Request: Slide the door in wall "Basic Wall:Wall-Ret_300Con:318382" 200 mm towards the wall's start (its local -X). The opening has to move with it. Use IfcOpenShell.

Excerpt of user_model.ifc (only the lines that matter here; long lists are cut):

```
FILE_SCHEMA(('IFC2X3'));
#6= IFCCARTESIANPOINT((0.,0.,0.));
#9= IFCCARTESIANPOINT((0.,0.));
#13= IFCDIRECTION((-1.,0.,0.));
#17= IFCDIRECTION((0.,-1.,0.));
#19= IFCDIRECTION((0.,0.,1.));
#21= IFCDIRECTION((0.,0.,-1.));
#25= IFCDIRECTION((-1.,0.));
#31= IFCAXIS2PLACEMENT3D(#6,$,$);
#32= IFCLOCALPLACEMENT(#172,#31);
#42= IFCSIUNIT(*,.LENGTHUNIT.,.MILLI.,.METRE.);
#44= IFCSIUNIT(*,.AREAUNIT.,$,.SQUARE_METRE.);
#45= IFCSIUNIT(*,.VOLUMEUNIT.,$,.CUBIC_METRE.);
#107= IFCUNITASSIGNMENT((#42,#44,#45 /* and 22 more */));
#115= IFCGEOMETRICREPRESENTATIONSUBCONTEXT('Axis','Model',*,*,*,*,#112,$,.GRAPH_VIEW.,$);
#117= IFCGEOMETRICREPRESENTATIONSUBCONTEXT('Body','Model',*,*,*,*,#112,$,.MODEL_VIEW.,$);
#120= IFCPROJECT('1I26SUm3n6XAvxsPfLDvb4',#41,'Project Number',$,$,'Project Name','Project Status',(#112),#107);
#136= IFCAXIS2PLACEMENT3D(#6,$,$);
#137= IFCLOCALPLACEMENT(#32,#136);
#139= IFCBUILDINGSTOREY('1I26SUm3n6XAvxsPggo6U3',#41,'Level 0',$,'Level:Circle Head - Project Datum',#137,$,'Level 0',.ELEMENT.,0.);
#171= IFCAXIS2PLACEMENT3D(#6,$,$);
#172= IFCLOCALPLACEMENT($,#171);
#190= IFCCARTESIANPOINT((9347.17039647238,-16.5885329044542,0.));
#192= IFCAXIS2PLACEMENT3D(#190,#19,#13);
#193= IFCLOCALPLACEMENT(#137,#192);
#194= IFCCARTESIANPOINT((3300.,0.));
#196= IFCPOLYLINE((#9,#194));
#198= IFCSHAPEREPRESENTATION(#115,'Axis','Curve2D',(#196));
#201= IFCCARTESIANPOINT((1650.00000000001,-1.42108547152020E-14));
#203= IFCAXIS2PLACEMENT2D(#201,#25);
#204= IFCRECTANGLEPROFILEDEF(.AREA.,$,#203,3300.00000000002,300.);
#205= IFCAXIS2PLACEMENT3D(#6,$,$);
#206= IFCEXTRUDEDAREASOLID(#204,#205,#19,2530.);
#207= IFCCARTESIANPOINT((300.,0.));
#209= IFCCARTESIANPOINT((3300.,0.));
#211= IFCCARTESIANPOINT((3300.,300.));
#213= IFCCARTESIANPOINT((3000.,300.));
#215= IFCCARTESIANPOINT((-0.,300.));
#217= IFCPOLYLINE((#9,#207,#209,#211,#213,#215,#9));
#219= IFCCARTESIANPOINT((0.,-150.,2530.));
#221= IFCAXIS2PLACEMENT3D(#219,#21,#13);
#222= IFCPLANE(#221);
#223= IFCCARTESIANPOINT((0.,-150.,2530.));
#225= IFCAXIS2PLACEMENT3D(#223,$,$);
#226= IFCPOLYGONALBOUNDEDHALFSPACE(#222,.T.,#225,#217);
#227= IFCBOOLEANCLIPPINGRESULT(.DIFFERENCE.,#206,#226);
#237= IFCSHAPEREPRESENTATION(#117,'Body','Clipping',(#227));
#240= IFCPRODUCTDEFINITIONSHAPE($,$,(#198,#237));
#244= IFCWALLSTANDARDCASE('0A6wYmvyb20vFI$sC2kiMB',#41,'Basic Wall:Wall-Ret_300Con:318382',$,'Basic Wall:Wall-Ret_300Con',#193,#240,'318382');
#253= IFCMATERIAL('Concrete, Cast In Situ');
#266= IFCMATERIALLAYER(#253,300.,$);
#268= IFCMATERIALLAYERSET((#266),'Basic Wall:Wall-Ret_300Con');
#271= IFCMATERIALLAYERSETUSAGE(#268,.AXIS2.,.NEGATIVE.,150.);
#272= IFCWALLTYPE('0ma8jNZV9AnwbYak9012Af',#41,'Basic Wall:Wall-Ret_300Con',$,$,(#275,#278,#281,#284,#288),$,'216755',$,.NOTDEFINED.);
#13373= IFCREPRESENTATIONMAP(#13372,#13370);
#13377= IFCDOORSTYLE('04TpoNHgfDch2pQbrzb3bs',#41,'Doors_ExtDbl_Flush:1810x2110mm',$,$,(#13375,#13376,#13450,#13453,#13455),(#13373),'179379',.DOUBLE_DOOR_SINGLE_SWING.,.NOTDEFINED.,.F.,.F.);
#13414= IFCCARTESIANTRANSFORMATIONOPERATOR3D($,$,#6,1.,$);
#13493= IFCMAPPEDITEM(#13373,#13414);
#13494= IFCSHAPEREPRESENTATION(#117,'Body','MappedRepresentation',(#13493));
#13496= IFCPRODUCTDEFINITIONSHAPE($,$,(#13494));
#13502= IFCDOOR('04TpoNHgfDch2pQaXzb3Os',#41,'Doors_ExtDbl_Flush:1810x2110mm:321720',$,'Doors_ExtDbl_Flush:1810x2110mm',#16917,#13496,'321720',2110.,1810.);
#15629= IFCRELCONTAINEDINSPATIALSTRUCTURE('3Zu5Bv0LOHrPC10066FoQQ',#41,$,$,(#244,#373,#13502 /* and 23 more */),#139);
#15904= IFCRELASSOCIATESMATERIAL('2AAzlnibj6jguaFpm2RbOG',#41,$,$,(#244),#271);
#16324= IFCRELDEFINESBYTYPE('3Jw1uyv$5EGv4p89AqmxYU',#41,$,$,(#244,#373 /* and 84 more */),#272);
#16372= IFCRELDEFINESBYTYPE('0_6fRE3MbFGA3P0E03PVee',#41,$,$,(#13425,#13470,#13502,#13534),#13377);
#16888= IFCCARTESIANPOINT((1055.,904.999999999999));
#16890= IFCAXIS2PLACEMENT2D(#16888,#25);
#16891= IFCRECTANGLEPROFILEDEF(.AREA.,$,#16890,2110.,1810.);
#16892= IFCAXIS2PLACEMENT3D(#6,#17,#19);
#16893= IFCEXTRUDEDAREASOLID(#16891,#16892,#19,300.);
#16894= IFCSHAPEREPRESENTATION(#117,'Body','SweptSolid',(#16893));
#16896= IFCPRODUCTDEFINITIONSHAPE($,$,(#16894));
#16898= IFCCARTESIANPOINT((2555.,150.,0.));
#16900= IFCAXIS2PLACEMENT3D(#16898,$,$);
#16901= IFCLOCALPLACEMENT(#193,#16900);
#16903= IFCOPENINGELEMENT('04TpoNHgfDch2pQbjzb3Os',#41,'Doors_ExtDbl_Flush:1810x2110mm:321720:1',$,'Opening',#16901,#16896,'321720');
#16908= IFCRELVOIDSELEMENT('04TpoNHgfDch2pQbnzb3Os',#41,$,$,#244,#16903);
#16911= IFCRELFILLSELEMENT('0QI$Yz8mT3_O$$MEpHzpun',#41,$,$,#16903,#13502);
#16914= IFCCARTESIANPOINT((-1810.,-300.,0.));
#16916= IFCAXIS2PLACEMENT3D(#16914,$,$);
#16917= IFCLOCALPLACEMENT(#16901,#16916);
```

```python
import ifcopenshell
import ifcopenshell.api.geometry
import ifcopenshell.util.placement
import ifcopenshell.util.unit

model = ifcopenshell.open("user_model.ifc")
unit_scale = ifcopenshell.util.unit.calculate_unit_scale(model)

door = model.by_id(13502)
opening = door.FillsVoids[0].RelatingOpeningElement
wall = opening.VoidsElements[0].RelatingBuildingElement

wall_matrix = ifcopenshell.util.placement.get_local_placement(wall.ObjectPlacement)
shift = wall_matrix[:3, 0] * -0.2 / unit_scale
before = ifcopenshell.util.placement.get_local_placement(door.ObjectPlacement)[:3, 3].copy()

# The door is placed relative to its opening, so it follows when the opening moves.
matrix = ifcopenshell.util.placement.get_local_placement(opening.ObjectPlacement)
matrix[:3, 3] += shift
ifcopenshell.api.geometry.edit_object_placement(
    model, product=opening, matrix=matrix, is_si=False, should_transform_children=True
)

after = ifcopenshell.util.placement.get_local_placement(door.ObjectPlacement)[:3, 3]
print("door moved by", (after - before).round(3) + 0.0)

model.write("user_model_edited.ifc")
```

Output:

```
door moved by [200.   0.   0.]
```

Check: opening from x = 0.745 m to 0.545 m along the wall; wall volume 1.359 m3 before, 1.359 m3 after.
